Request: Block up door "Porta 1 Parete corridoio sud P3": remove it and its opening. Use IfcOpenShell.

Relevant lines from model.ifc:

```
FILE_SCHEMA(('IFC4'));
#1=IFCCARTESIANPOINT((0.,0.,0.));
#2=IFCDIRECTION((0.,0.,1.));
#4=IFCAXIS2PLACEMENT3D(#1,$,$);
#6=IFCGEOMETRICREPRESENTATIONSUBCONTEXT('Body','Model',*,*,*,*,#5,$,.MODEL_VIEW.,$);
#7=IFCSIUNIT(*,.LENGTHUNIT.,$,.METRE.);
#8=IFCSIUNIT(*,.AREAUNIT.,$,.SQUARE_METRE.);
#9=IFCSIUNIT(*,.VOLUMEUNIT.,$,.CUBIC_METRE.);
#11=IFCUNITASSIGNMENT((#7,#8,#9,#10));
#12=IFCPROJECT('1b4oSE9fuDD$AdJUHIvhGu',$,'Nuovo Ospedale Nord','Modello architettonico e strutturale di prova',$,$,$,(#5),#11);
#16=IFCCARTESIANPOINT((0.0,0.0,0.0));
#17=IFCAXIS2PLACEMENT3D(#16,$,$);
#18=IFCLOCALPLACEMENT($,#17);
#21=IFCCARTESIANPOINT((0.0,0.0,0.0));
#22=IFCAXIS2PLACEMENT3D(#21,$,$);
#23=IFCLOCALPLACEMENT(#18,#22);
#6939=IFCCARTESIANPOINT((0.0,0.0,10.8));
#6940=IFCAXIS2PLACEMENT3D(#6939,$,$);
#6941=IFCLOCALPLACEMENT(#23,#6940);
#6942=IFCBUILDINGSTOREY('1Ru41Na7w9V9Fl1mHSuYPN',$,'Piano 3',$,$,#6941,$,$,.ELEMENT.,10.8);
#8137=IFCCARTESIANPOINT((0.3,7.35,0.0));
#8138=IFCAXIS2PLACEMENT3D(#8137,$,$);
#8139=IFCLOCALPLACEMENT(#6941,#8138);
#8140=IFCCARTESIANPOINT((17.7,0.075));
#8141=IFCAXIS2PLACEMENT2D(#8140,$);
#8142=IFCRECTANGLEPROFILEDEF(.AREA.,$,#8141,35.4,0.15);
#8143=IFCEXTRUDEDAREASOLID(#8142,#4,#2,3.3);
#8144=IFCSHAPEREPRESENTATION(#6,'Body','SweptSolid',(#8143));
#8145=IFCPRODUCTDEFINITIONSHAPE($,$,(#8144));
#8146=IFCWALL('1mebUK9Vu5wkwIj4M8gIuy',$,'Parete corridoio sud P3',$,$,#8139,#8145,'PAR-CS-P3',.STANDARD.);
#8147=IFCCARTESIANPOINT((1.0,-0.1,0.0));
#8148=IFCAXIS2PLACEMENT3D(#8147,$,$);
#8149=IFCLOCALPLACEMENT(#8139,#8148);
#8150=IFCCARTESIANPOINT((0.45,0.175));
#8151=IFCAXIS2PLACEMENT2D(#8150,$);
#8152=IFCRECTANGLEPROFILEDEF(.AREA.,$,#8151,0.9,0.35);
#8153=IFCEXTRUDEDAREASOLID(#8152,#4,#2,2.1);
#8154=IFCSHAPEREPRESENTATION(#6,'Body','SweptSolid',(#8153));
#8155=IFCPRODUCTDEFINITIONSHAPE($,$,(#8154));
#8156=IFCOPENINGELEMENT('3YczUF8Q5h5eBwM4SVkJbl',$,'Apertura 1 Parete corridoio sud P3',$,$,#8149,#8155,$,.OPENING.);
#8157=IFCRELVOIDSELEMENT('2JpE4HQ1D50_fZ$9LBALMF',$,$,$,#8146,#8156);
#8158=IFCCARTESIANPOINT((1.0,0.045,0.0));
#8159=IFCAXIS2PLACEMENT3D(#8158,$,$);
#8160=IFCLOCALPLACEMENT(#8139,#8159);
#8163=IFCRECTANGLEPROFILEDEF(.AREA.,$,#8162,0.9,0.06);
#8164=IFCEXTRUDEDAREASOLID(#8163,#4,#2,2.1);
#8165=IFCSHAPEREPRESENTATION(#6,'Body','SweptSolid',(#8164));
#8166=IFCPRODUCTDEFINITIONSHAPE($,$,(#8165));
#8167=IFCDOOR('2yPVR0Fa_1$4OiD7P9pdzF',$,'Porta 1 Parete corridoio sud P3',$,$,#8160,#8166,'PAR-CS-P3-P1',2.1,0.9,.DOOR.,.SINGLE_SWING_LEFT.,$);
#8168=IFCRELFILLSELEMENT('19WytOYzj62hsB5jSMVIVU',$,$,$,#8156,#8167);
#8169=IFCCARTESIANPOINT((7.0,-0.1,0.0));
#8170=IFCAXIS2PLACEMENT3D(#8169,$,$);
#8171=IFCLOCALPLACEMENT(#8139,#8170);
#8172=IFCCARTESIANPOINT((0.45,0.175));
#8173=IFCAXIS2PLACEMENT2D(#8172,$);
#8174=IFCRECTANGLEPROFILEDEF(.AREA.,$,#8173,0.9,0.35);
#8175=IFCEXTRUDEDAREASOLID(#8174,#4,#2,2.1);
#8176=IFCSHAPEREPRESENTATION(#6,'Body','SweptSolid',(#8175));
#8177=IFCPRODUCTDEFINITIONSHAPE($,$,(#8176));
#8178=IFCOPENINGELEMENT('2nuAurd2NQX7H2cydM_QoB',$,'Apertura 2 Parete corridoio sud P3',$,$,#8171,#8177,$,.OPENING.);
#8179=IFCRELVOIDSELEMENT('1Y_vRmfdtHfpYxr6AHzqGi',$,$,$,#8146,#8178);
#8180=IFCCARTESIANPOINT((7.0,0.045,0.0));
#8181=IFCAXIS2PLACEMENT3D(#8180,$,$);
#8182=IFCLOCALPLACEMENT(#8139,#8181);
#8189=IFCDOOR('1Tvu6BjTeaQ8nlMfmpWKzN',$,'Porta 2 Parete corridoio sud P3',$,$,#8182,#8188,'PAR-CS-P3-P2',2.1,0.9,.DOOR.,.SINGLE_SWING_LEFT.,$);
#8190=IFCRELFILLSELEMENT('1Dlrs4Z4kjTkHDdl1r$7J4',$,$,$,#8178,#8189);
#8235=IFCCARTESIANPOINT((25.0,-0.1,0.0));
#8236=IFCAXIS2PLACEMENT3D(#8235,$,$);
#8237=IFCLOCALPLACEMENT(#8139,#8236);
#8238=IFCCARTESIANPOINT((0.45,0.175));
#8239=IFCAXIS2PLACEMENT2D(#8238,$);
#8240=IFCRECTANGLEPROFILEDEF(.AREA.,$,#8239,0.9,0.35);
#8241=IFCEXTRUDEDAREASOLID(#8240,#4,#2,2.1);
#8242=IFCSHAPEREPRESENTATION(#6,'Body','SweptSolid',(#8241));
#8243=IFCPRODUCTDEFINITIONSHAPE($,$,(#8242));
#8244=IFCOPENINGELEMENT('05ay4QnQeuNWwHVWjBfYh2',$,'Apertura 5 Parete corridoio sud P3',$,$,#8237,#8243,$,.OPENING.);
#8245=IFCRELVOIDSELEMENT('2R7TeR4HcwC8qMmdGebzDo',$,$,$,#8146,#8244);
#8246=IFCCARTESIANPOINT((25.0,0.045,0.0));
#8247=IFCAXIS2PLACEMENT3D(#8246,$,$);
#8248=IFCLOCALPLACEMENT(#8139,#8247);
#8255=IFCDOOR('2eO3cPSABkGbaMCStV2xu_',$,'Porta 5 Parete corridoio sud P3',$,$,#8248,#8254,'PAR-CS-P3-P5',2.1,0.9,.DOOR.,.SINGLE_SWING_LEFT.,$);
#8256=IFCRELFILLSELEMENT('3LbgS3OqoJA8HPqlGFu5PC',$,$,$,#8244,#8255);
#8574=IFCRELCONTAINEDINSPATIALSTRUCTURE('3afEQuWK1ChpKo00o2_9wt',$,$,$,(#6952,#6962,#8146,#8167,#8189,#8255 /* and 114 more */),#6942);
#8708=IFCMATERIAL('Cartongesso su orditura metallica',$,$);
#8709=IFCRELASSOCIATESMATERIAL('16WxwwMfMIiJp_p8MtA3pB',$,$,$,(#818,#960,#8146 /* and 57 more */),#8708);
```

```python
import ifcopenshell
import ifcopenshell.api.feature
import ifcopenshell.api.root
import ifcopenshell.geom
import ifcopenshell.util.shape

model = ifcopenshell.open("model.ifc")
settings = ifcopenshell.geom.settings()


def volume(element):
    """Net volume in cubic metres, openings subtracted."""
    shape = ifcopenshell.geom.create_shape(settings, element)
    return ifcopenshell.util.shape.get_volume(shape.geometry)


door = model.by_guid("2yPVR0Fa_1$4OiD7P9pdzF")
opening = door.FillsVoids[0].RelatingOpeningElement
wall = opening.VoidsElements[0].RelatingBuildingElement
before = volume(wall)

ifcopenshell.api.root.remove_product(model, product=door)
ifcopenshell.api.feature.remove_feature(model, feature=opening)

after = volume(wall)

print(f"wall volume {before:.3f} -> {after:.3f} m3")

model.write("model_v2.ifc")
```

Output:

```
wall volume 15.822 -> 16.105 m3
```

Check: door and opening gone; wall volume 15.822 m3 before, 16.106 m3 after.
